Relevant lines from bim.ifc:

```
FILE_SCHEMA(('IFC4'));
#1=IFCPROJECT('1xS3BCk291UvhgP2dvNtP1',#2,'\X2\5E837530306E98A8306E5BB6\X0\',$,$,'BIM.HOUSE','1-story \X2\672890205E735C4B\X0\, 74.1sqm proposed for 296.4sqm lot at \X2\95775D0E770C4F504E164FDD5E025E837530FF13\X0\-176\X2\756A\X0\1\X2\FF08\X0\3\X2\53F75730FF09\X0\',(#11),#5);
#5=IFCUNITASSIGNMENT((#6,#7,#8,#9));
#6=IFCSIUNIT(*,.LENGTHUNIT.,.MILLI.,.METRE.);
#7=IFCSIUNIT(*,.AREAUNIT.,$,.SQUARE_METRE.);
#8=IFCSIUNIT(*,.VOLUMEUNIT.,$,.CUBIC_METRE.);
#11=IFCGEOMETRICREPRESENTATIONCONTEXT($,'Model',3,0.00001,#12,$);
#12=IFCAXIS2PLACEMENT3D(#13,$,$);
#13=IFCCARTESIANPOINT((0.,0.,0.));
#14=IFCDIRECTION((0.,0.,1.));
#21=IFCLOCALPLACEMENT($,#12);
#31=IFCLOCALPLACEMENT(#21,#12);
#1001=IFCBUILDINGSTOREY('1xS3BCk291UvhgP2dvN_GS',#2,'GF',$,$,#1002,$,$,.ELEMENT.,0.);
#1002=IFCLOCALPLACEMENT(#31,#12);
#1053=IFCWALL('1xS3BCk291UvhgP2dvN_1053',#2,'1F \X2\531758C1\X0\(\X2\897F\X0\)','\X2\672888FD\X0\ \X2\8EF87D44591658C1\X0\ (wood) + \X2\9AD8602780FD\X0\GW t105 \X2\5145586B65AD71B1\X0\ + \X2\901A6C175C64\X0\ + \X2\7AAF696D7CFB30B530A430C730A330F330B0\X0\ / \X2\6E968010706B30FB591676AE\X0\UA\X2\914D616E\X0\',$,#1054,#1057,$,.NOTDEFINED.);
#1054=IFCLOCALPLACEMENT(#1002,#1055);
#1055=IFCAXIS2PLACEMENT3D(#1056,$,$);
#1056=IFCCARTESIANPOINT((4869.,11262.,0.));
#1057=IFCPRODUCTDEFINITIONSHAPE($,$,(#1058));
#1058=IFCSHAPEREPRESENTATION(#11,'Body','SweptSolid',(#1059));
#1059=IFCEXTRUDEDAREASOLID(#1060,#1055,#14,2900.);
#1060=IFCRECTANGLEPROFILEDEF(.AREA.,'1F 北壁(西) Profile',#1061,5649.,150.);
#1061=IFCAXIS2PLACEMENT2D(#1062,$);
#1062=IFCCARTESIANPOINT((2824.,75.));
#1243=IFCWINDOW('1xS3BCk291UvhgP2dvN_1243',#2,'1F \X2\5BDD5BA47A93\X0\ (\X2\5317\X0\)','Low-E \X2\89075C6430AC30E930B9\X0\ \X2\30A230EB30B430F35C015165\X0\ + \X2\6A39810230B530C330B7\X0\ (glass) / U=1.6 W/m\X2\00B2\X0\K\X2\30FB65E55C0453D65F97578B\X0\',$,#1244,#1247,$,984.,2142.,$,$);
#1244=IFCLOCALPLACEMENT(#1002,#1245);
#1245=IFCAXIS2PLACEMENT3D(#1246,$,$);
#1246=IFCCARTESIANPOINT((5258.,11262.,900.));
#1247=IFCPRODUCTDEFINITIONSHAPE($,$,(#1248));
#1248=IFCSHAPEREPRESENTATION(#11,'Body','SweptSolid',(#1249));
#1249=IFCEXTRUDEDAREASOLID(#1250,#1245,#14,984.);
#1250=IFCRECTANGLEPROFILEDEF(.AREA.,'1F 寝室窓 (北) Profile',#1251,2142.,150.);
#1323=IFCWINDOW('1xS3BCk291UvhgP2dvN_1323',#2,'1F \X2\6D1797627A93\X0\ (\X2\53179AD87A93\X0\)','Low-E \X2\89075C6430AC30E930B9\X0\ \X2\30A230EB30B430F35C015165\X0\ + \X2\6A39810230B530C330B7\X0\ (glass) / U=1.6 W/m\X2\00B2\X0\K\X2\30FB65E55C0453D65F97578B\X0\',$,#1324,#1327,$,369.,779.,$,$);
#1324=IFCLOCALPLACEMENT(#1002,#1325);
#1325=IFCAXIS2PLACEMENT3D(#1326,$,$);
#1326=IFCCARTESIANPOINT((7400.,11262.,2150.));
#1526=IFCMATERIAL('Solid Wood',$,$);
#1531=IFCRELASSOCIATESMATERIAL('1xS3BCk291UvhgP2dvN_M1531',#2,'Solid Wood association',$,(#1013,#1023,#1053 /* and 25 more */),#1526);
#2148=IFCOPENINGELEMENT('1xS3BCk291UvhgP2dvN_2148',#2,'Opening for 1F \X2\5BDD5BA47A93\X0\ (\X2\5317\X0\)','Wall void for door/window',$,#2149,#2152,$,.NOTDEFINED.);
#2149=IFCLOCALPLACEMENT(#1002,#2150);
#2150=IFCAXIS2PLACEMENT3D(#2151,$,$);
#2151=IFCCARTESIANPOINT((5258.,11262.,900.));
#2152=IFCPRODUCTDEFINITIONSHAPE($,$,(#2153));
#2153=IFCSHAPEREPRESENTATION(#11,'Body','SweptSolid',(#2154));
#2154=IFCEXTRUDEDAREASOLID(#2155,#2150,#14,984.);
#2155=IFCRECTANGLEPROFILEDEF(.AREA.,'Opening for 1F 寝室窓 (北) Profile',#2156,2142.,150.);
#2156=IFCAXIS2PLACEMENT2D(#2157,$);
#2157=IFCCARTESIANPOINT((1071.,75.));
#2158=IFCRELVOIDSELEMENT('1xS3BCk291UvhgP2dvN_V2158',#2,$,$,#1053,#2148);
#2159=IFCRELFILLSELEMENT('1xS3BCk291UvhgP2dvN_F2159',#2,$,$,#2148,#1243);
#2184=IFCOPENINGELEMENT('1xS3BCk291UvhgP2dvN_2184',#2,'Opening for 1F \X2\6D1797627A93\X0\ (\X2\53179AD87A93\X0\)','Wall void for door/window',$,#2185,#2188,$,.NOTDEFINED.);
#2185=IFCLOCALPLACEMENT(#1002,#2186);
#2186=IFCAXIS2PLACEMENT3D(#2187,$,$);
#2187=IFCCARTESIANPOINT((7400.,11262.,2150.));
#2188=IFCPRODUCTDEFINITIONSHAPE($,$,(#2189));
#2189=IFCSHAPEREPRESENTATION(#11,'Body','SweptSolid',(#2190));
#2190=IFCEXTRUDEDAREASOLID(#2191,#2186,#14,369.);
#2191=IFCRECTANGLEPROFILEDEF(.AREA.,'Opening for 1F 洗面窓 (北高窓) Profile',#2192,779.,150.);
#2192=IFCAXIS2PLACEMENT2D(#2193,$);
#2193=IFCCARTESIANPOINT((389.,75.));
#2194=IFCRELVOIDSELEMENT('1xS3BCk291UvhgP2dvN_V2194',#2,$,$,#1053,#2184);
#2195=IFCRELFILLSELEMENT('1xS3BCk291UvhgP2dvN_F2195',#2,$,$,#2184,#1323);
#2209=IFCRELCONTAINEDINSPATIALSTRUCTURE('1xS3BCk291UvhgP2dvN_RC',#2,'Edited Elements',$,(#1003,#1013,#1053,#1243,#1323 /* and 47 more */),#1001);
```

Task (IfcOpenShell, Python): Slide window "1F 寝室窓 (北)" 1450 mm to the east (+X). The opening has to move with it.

```python
import ifcopenshell
import ifcopenshell.api.geometry
import ifcopenshell.util.placement
import ifcopenshell.util.unit

model = ifcopenshell.open("bim.ifc")
unit_scale = ifcopenshell.util.unit.calculate_unit_scale(model)

window = model.by_guid("1xS3BCk291UvhgP2dvN_1243")
opening = window.FillsVoids[0].RelatingOpeningElement
wall = opening.VoidsElements[0].RelatingBuildingElement

wall_matrix = ifcopenshell.util.placement.get_local_placement(wall.ObjectPlacement)
shift = wall_matrix[:3, 0] * 1.45 / unit_scale
before = ifcopenshell.util.placement.get_local_placement(window.ObjectPlacement)[:3, 3].copy()

# The window is not placed relative to its opening, so move both.
for product in (opening, window):
    matrix = ifcopenshell.util.placement.get_local_placement(product.ObjectPlacement)
    matrix[:3, 3] += shift
    ifcopenshell.api.geometry.edit_object_placement(model, product=product, matrix=matrix, is_si=False)

after = ifcopenshell.util.placement.get_local_placement(window.ObjectPlacement)[:3, 3]
print("window moved by", (after - before).round(3) + 0.0)

model.write("bim_edited.ifc")
```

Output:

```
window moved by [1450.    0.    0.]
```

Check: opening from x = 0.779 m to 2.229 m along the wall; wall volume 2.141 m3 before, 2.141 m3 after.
